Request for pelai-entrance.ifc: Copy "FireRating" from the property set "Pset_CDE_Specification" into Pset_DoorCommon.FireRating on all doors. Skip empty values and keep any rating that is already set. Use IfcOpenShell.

First a look at what the model holds.

```python
import ifcopenshell
import ifcopenshell.util.element

model = ifcopenshell.open("pelai-entrance.ifc")
print(model.schema)
doors = model.by_type("IfcDoor")
print(len(doors), "doors")
for e in doors[:8]:
    source = ifcopenshell.util.element.get_pset(e, "Pset_CDE_Specification", "FireRating")
    target = ifcopenshell.util.element.get_pset(e, "Pset_DoorCommon", "FireRating")
    print(e.id(), repr(source), repr(target), sep=" | ")
```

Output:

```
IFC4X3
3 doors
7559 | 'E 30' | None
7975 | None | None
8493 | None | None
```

```python
import ifcopenshell
import ifcopenshell.api.pset
import ifcopenshell.util.element

model = ifcopenshell.open("pelai-entrance.ifc")

count = 0
for e in model.by_type("IfcDoor"):
    value = ifcopenshell.util.element.get_pset(e, "Pset_CDE_Specification", "FireRating")
    current = ifcopenshell.util.element.get_pset(e, "Pset_DoorCommon", "FireRating")
    if not value or not value.strip() or current:
        continue
    # add_pset returns the element's existing set when there is one.
    pset = ifcopenshell.api.pset.add_pset(model, product=e, name="Pset_DoorCommon")
    ifcopenshell.api.pset.edit_pset(model, pset=pset, properties={"FireRating": value})
    count += 1

print(count, "doors updated")

model.write("pelai-entrance-out.ifc")
```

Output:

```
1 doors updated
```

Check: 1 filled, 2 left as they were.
